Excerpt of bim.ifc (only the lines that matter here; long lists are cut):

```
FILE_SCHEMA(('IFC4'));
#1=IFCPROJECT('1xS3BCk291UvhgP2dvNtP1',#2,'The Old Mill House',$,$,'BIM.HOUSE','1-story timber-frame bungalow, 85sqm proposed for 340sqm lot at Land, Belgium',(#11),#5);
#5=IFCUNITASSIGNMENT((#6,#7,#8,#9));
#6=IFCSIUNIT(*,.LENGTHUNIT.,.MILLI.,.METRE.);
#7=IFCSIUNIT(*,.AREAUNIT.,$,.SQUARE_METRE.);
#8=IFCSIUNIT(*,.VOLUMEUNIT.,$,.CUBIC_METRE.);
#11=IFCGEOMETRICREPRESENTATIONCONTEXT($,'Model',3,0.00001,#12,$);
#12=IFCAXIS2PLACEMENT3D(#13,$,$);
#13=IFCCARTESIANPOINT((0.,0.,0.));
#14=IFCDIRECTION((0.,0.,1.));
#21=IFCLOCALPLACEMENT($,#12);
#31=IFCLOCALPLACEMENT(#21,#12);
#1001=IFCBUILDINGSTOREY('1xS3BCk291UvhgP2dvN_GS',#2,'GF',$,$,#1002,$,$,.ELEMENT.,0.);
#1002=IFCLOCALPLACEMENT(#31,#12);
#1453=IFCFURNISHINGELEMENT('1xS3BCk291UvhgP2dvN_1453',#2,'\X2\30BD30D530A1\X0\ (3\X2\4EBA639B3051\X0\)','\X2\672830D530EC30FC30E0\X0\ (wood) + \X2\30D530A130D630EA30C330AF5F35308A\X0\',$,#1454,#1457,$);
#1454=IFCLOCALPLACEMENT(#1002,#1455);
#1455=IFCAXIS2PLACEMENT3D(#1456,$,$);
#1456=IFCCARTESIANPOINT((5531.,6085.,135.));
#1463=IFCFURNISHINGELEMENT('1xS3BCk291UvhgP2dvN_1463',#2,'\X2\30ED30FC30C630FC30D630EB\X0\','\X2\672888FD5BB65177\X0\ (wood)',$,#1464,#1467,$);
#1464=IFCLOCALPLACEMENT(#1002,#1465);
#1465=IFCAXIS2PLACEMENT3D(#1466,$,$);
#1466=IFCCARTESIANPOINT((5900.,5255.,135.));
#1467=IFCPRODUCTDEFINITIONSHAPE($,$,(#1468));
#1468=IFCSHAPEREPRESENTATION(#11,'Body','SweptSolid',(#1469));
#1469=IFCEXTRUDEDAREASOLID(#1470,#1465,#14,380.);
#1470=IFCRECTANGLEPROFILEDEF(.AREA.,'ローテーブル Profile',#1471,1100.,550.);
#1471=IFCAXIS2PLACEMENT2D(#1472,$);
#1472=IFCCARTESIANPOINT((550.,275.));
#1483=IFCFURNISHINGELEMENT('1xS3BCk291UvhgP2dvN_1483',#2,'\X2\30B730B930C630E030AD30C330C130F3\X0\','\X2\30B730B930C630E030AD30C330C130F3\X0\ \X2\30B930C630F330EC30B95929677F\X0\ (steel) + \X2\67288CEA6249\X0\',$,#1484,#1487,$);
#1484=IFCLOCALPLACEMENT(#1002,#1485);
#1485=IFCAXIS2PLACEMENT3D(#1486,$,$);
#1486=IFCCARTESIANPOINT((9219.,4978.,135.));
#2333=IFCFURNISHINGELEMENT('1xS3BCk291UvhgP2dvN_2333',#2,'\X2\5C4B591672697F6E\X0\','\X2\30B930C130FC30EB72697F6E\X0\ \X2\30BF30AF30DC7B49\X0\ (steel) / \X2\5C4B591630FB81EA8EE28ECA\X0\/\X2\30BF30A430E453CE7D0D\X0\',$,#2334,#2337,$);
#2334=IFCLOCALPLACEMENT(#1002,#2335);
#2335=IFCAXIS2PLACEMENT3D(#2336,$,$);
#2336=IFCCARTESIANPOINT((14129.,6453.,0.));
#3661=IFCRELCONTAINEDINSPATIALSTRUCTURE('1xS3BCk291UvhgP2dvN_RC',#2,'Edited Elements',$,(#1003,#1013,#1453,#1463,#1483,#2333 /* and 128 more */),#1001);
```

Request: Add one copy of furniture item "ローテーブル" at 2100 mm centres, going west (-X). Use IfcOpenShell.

```python
import numpy as np
import ifcopenshell
import ifcopenshell.api.geometry
import ifcopenshell.api.root
import ifcopenshell.util.element
import ifcopenshell.util.placement
import ifcopenshell.util.unit

model = ifcopenshell.open("bim.ifc")
unit_scale = ifcopenshell.util.unit.calculate_unit_scale(model)


def reuse_history(source, copy):
    """copy_class also copies each property set's owner history, people and application; keep the originals."""
    for rel in copy.IsDefinedBy:
        if rel.is_a("IfcRelDefinesByProperties") and (history := rel.RelatingPropertyDefinition.OwnerHistory):
            rel.RelatingPropertyDefinition.OwnerHistory = source.OwnerHistory
            ifcopenshell.util.element.remove_deep2(model, history)


source = model.by_guid("1xS3BCk291UvhgP2dvN_1463")
base = ifcopenshell.util.placement.get_local_placement(source.ObjectPlacement)
step = np.array([-1.0, 0.0, 0.0]) * 2.1 / unit_scale

for i in range(1, 2):
    copy = ifcopenshell.api.root.copy_class(model, product=source)
    copy.Representation = ifcopenshell.util.element.copy_deep(
        model, source.Representation, exclude=["IfcGeometricRepresentationContext", "IfcRepresentationMap"]
    )
    reuse_history(source, copy)
    matrix = base.copy()
    matrix[:3, 3] += i * step
    print("added at", matrix[:3, 3].round(3) + 0.0)
    ifcopenshell.api.geometry.edit_object_placement(model, product=copy, matrix=matrix, is_si=False)

model.write("bim_edited.ifc")
```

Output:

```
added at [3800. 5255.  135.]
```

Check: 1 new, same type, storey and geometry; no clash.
